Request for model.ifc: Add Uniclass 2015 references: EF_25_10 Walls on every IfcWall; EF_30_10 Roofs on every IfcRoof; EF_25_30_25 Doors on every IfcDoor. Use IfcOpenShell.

First a look at what the model holds.

```python
import ifcopenshell

model = ifcopenshell.open("model.ifc")
print(model.schema)
print("classifications:", [c.Name for c in model.by_type("IfcClassification")])
for ifc_class in ("IfcDoor", "IfcRoof", "IfcStair", "IfcWall", "IfcWindow"):
    print(ifc_class, len(model.by_type(ifc_class)))
```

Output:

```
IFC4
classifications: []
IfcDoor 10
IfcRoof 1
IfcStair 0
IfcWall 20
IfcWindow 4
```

```python
import ifcopenshell
import ifcopenshell.api.classification

model = ifcopenshell.open("model.ifc")

system = ifcopenshell.api.classification.add_classification(model, classification="Uniclass 2015")

codes = {
    "IfcWall": ("EF_25_10", "Walls"),
    "IfcRoof": ("EF_30_10", "Roofs"),
    "IfcDoor": ("EF_25_30_25", "Doors"),
}
for ifc_class, (code, name) in codes.items():
    products = model.by_type(ifc_class)
    ifcopenshell.api.classification.add_reference(
        model, products=products, classification=system, identification=code, name=name
    )
    print(code, len(products))

model.write("model_edited.ifc")
```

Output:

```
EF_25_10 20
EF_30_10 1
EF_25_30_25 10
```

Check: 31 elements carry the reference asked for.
